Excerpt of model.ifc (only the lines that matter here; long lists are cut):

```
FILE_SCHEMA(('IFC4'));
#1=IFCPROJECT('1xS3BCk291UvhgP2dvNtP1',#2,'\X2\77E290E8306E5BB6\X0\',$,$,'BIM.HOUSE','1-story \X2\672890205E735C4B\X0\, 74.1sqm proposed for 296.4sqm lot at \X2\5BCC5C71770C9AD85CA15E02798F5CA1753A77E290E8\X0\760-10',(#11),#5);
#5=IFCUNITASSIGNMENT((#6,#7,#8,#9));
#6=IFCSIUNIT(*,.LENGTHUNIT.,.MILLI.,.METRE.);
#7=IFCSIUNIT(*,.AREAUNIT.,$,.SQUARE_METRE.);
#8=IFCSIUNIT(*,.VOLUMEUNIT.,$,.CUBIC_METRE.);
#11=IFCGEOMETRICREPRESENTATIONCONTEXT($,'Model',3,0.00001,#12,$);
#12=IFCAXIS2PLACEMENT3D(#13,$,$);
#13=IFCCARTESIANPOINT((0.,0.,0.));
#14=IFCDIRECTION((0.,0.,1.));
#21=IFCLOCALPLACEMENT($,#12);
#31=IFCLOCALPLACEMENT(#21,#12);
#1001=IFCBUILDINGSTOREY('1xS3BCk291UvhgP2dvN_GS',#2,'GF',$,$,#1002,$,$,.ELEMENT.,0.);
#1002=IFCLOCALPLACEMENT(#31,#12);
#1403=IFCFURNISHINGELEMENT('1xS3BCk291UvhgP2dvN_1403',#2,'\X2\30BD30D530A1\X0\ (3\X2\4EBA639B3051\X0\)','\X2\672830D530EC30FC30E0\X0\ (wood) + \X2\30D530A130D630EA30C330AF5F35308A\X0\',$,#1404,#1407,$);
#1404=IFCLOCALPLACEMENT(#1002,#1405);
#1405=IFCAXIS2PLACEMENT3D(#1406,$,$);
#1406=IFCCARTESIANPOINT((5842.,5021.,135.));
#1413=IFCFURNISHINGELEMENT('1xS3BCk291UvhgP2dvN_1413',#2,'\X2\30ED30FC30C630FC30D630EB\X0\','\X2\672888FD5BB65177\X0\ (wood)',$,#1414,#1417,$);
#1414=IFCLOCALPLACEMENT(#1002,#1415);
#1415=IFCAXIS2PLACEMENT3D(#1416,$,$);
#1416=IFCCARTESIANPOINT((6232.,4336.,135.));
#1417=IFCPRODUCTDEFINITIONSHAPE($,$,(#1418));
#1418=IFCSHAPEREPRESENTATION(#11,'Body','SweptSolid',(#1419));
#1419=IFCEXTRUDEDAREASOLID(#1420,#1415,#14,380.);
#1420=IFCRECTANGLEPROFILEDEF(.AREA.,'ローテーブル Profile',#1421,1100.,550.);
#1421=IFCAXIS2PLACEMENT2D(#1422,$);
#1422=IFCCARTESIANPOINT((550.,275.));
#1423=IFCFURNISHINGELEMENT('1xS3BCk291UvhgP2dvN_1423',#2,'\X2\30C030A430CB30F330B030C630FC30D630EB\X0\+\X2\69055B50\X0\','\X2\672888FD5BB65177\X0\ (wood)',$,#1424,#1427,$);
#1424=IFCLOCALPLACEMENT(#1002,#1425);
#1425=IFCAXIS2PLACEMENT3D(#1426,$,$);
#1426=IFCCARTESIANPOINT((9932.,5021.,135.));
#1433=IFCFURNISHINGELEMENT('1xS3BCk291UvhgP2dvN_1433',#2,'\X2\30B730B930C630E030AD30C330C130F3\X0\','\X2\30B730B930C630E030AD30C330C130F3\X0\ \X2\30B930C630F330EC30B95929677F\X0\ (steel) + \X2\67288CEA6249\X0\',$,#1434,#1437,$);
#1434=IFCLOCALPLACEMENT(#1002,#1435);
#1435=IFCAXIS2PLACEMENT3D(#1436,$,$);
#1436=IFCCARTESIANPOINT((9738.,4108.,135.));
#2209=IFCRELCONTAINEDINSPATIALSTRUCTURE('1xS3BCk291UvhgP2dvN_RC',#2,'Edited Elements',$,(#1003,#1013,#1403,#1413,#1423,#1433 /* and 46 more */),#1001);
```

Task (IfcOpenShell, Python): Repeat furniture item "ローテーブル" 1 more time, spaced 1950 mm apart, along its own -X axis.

```python
import ifcopenshell
import ifcopenshell.api.geometry
import ifcopenshell.api.root
import ifcopenshell.util.element
import ifcopenshell.util.placement
import ifcopenshell.util.unit

model = ifcopenshell.open("model.ifc")
unit_scale = ifcopenshell.util.unit.calculate_unit_scale(model)


def reuse_history(source, copy):
    """copy_class also copies each property set's owner history, people and application; keep the originals."""
    for rel in copy.IsDefinedBy:
        if rel.is_a("IfcRelDefinesByProperties") and (history := rel.RelatingPropertyDefinition.OwnerHistory):
            rel.RelatingPropertyDefinition.OwnerHistory = source.OwnerHistory
            ifcopenshell.util.element.remove_deep2(model, history)


source = model.by_id(1413)
base = ifcopenshell.util.placement.get_local_placement(source.ObjectPlacement)
step = -base[:3, 0] * 1.95 / unit_scale

for i in range(1, 2):
    copy = ifcopenshell.api.root.copy_class(model, product=source)
    copy.Representation = ifcopenshell.util.element.copy_deep(
        model, source.Representation, exclude=["IfcGeometricRepresentationContext", "IfcRepresentationMap"]
    )
    reuse_history(source, copy)
    matrix = base.copy()
    matrix[:3, 3] += i * step
    print("added at", matrix[:3, 3].round(3) + 0.0)
    ifcopenshell.api.geometry.edit_object_placement(model, product=copy, matrix=matrix, is_si=False)

model.write("model-out.ifc")
```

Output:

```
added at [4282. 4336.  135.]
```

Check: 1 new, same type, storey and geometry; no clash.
